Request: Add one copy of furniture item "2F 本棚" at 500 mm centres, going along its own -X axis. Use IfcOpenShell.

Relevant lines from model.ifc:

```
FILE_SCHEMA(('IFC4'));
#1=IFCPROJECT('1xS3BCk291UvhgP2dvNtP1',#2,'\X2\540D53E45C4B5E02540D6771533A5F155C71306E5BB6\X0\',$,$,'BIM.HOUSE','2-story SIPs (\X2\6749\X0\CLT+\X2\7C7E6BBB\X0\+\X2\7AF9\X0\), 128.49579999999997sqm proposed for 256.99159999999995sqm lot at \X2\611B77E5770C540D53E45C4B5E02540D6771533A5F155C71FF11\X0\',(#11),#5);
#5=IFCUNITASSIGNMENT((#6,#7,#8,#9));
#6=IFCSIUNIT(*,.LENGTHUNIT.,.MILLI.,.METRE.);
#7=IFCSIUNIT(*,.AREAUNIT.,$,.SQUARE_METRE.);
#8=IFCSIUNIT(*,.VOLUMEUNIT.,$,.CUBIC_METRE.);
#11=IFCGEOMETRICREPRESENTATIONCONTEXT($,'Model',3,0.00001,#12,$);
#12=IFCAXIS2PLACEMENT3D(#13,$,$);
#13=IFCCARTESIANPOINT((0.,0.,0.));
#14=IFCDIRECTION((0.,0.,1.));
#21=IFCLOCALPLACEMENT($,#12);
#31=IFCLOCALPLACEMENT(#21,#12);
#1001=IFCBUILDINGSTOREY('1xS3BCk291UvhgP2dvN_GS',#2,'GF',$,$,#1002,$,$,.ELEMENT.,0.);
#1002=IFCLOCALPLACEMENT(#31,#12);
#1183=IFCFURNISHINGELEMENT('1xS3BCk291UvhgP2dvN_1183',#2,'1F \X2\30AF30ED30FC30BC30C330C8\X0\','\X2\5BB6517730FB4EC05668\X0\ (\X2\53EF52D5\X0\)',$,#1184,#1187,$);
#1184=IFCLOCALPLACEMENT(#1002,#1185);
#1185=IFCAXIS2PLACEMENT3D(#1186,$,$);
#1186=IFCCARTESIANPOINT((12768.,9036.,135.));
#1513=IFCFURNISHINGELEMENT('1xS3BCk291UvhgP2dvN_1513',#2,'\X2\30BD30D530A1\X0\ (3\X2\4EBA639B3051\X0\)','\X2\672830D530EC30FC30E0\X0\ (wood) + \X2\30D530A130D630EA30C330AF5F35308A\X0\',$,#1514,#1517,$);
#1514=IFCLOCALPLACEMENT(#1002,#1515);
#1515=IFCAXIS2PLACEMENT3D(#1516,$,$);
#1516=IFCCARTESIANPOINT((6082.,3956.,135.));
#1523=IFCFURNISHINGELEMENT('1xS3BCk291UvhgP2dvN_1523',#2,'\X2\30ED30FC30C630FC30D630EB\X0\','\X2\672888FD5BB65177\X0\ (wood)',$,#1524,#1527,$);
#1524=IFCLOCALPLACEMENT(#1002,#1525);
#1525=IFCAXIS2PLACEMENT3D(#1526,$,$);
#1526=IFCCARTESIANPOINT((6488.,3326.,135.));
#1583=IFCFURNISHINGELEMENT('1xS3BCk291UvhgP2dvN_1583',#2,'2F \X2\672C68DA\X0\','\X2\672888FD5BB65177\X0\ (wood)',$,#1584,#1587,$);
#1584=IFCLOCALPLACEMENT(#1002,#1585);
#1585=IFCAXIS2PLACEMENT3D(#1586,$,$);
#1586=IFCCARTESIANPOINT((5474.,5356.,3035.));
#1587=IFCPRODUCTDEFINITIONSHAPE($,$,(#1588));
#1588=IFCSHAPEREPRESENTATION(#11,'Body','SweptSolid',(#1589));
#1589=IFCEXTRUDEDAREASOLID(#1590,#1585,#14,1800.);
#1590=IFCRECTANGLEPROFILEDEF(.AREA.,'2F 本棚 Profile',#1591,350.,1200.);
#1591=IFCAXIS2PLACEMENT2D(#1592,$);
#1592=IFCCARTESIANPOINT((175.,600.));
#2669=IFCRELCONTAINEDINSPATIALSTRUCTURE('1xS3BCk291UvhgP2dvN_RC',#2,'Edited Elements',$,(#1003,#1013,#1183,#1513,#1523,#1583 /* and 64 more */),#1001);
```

```python
import ifcopenshell
import ifcopenshell.api.geometry
import ifcopenshell.api.root
import ifcopenshell.util.element
import ifcopenshell.util.placement
import ifcopenshell.util.unit

model = ifcopenshell.open("model.ifc")
unit_scale = ifcopenshell.util.unit.calculate_unit_scale(model)


def reuse_history(source, copy):
    """copy_class also copies each property set's owner history, people and application; keep the originals."""
    for rel in copy.IsDefinedBy:
        if rel.is_a("IfcRelDefinesByProperties") and (history := rel.RelatingPropertyDefinition.OwnerHistory):
            rel.RelatingPropertyDefinition.OwnerHistory = source.OwnerHistory
            ifcopenshell.util.element.remove_deep2(model, history)


source = model.by_id(1583)
base = ifcopenshell.util.placement.get_local_placement(source.ObjectPlacement)
step = -base[:3, 0] * 0.5 / unit_scale

for i in range(1, 2):
    copy = ifcopenshell.api.root.copy_class(model, product=source)
    copy.Representation = ifcopenshell.util.element.copy_deep(
        model, source.Representation, exclude=["IfcGeometricRepresentationContext", "IfcRepresentationMap"]
    )
    reuse_history(source, copy)
    matrix = base.copy()
    matrix[:3, 3] += i * step
    print("added at", matrix[:3, 3].round(3) + 0.0)
    ifcopenshell.api.geometry.edit_object_placement(model, product=copy, matrix=matrix, is_si=False)

model.write("model_rev.ifc")
```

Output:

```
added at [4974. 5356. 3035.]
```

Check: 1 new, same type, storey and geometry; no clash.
